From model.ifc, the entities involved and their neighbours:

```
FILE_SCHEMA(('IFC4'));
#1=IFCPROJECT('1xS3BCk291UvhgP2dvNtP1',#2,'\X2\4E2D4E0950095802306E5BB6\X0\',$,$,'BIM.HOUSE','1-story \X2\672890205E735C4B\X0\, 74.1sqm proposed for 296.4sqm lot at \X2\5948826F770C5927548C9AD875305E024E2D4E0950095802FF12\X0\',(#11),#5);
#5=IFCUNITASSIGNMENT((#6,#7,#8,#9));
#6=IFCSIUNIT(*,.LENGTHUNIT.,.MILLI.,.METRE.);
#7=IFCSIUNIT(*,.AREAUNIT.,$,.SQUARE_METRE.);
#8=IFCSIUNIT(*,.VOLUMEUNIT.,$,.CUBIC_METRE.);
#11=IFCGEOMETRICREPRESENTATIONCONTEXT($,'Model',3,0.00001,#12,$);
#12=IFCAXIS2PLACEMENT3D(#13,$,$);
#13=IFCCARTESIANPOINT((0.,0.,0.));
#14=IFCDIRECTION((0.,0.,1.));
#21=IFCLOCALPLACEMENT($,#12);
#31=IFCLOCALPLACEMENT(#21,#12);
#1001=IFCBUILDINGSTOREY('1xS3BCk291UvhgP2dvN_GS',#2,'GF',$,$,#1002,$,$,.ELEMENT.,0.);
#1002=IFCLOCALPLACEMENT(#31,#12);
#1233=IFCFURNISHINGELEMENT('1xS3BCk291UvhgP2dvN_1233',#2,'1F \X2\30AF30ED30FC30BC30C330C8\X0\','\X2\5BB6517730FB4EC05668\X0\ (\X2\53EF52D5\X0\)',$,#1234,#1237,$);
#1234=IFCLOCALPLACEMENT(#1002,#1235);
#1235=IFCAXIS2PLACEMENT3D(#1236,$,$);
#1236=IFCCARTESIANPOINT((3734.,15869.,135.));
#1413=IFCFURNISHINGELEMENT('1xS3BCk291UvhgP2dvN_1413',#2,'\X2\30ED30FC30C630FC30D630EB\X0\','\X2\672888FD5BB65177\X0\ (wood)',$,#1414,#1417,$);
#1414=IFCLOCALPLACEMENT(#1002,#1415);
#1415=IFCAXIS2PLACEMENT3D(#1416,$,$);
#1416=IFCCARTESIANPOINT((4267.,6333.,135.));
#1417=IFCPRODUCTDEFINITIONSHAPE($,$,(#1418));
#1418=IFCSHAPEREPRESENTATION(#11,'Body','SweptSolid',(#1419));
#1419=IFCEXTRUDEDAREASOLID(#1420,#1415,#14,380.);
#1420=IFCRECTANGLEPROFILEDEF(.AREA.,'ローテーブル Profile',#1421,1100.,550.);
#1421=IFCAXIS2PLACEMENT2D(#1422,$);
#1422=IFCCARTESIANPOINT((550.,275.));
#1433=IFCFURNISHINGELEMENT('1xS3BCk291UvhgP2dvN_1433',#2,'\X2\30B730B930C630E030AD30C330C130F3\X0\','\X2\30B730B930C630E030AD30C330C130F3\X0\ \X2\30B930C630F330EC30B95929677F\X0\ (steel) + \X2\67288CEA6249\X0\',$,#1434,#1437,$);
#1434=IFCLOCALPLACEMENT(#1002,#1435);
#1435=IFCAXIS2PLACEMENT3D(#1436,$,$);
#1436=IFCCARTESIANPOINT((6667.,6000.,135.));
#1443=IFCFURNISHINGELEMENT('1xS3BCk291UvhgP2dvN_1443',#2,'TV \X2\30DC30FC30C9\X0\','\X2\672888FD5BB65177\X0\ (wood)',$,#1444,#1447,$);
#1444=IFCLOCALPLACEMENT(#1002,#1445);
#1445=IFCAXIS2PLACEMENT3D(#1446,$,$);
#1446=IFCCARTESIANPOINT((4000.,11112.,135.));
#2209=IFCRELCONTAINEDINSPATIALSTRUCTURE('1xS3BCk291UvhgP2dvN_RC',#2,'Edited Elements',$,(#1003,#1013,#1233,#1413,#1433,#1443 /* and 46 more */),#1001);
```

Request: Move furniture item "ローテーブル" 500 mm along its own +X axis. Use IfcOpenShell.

```python
import ifcopenshell
import ifcopenshell.api.geometry
import ifcopenshell.util.placement
import ifcopenshell.util.unit

model = ifcopenshell.open("model.ifc")
unit_scale = ifcopenshell.util.unit.calculate_unit_scale(model)

item = model.by_id(1413)
matrix = ifcopenshell.util.placement.get_local_placement(item.ObjectPlacement)
matrix[:3, 3] += matrix[:3, 0] * 0.5 / unit_scale
ifcopenshell.api.geometry.edit_object_placement(model, product=item, matrix=matrix, is_si=False)

print(ifcopenshell.util.placement.get_local_placement(item.ObjectPlacement).round(3) + 0.0)

model.write("model_updated.ifc")
```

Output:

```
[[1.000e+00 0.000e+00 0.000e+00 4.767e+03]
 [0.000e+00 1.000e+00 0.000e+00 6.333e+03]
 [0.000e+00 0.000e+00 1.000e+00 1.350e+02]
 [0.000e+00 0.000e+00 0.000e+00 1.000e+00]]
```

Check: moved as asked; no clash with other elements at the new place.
